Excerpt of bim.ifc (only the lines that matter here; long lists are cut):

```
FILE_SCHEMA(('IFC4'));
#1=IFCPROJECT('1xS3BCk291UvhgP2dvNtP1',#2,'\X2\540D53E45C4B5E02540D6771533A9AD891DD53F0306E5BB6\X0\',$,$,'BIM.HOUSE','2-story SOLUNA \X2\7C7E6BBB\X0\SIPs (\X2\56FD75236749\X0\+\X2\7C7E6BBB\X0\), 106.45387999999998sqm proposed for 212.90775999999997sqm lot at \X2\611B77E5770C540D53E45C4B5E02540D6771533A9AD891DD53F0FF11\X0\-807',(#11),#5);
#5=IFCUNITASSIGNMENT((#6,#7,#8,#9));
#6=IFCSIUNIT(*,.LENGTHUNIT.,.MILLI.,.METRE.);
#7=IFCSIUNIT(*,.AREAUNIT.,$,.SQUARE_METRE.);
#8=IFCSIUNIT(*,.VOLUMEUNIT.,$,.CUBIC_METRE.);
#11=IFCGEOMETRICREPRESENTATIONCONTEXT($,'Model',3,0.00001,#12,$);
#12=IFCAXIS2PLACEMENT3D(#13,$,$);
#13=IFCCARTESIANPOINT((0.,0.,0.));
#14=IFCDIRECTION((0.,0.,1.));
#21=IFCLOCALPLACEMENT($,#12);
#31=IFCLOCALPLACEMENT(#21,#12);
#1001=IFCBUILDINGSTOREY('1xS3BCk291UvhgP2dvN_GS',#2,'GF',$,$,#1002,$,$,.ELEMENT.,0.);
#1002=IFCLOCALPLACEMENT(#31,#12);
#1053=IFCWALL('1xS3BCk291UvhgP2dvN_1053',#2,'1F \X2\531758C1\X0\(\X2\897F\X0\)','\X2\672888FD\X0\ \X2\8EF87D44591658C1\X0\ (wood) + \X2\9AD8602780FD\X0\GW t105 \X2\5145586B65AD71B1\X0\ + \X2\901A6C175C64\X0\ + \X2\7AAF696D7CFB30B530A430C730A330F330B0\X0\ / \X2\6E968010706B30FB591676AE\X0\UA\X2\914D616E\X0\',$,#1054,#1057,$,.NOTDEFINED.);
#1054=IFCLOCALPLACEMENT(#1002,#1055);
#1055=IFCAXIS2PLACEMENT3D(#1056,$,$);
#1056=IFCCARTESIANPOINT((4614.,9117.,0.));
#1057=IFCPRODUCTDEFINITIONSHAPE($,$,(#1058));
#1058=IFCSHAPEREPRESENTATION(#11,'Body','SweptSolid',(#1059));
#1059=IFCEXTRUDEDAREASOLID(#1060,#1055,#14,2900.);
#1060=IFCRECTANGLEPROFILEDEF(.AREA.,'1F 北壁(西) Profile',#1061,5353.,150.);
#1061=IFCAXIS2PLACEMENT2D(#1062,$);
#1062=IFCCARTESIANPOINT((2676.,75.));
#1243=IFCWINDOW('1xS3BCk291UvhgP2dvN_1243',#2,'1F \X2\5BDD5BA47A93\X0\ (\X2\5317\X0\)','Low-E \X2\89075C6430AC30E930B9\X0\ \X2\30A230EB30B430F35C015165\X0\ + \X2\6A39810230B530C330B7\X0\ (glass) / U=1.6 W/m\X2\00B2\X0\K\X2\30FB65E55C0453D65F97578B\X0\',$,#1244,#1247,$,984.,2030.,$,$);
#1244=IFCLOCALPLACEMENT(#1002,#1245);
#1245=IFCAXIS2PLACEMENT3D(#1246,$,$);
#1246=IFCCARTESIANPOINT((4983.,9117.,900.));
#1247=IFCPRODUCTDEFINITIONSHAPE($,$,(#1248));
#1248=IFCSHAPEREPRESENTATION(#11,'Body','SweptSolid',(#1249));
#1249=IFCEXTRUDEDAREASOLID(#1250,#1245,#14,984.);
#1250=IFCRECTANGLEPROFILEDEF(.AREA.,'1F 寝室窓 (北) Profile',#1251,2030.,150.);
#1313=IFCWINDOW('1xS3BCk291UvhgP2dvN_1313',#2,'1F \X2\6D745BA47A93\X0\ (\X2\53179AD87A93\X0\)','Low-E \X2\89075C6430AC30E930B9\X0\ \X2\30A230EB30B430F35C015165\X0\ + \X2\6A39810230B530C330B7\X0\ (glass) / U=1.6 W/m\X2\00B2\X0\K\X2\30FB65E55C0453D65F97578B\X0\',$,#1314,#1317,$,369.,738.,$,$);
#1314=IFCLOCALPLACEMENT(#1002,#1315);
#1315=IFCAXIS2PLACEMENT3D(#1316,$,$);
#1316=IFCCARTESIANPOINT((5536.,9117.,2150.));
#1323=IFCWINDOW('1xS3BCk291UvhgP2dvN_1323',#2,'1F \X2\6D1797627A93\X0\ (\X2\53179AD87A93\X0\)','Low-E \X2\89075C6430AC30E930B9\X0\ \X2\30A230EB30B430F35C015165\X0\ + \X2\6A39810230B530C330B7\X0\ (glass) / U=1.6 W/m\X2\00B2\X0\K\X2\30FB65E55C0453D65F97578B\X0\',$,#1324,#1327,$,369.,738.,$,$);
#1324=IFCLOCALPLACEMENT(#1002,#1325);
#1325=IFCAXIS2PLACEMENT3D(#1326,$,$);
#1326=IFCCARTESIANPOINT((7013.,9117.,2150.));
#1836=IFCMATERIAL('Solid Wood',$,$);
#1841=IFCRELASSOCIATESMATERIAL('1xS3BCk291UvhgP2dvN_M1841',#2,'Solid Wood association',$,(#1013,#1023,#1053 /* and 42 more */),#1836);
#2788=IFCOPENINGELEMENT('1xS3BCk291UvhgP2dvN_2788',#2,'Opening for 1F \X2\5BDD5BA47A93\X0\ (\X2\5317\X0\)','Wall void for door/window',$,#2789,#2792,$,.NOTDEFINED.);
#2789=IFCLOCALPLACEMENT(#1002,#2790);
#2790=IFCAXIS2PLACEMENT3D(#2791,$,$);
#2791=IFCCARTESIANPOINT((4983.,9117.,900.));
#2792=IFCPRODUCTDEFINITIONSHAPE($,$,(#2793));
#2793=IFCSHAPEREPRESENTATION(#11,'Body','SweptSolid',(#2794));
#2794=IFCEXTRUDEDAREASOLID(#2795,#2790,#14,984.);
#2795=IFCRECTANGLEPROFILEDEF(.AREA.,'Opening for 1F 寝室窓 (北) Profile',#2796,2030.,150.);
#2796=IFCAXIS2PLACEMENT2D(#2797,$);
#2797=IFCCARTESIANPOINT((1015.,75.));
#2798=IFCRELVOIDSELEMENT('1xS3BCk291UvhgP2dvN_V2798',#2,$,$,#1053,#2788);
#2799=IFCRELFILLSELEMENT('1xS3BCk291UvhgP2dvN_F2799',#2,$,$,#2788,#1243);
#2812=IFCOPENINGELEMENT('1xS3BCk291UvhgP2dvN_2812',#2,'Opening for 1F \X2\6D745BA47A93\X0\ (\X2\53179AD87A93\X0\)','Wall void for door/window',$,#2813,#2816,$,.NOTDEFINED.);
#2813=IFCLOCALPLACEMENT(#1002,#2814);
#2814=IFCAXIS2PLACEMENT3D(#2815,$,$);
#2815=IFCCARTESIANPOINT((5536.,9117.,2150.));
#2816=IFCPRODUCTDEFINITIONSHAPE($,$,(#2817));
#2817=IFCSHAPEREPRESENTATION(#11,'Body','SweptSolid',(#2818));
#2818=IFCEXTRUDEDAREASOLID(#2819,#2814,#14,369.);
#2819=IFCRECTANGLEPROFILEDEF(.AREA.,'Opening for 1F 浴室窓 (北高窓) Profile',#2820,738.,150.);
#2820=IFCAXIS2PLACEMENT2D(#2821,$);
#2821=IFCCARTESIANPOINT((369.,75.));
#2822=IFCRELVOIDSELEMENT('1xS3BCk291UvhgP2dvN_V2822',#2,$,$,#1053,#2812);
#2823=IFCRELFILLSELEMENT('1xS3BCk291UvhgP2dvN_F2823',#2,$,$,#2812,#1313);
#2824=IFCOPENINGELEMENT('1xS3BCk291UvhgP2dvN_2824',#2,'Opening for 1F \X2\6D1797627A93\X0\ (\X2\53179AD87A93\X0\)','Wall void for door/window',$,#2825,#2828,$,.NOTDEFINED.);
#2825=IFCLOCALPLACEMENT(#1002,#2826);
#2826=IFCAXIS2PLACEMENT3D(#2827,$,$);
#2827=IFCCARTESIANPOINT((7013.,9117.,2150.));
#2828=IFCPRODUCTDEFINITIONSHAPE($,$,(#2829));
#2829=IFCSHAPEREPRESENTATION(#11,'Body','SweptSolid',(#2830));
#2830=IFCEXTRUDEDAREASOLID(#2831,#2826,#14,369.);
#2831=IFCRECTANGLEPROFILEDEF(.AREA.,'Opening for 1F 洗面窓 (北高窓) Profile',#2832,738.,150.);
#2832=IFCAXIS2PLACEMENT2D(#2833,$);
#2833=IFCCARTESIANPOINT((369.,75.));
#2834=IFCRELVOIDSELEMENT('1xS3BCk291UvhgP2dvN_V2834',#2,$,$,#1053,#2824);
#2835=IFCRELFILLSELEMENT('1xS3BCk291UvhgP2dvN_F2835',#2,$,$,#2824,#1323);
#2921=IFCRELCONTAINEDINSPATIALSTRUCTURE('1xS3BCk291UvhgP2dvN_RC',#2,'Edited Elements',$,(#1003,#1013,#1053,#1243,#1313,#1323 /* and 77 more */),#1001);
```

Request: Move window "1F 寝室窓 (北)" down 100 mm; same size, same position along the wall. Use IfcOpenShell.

```python
import numpy as np
import ifcopenshell
import ifcopenshell.api.geometry
import ifcopenshell.util.placement
import ifcopenshell.util.unit

model = ifcopenshell.open("bim.ifc")
unit_scale = ifcopenshell.util.unit.calculate_unit_scale(model)

window = model.by_id(1243)
opening = window.FillsVoids[0].RelatingOpeningElement
dz = -100.0

shift = np.array([0.0, 0.0, dz])
# The window is not placed relative to its opening, so move both.
for product in (opening, window):
    matrix = ifcopenshell.util.placement.get_local_placement(product.ObjectPlacement)
    matrix[:3, 3] += shift
    ifcopenshell.api.geometry.edit_object_placement(model, product=product, matrix=matrix, is_si=False)

print(f"moved by {dz * unit_scale:+.3f} m")

model.write("bim_rev.ifc")
```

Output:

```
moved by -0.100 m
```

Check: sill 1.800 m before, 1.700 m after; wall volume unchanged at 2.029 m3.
